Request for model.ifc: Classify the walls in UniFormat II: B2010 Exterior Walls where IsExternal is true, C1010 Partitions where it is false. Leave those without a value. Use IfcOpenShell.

First a look at what the model holds.

```python
import ifcopenshell
import ifcopenshell.util.element

model = ifcopenshell.open("model.ifc")
print(model.schema)
print("classifications:", [c.Name for c in model.by_type("IfcClassification")])
values = [ifcopenshell.util.element.get_pset(e, "Pset_WallCommon", "IsExternal") for e in model.by_type("IfcWall")]
for value in (True, False, None):
    print("IsExternal", value, values.count(value))
```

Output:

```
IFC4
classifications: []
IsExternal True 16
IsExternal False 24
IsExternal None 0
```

```python
import ifcopenshell
import ifcopenshell.api.classification
import ifcopenshell.util.element

model = ifcopenshell.open("model.ifc")

system = ifcopenshell.api.classification.add_classification(model, classification="UniFormat II")

walls = model.by_type("IfcWall")
external = {e: ifcopenshell.util.element.get_pset(e, "Pset_WallCommon", "IsExternal") for e in walls}
for flag, code, name in ((True, "B2010", "Exterior Walls"), (False, "C1010", "Partitions")):
    products = [e for e in walls if external[e] is flag]
    ifcopenshell.api.classification.add_reference(
        model, products=products, classification=system, identification=code, name=name
    )
    print(code, len(products))

model.write("model_rev.ifc")
```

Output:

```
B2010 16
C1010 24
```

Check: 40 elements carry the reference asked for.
